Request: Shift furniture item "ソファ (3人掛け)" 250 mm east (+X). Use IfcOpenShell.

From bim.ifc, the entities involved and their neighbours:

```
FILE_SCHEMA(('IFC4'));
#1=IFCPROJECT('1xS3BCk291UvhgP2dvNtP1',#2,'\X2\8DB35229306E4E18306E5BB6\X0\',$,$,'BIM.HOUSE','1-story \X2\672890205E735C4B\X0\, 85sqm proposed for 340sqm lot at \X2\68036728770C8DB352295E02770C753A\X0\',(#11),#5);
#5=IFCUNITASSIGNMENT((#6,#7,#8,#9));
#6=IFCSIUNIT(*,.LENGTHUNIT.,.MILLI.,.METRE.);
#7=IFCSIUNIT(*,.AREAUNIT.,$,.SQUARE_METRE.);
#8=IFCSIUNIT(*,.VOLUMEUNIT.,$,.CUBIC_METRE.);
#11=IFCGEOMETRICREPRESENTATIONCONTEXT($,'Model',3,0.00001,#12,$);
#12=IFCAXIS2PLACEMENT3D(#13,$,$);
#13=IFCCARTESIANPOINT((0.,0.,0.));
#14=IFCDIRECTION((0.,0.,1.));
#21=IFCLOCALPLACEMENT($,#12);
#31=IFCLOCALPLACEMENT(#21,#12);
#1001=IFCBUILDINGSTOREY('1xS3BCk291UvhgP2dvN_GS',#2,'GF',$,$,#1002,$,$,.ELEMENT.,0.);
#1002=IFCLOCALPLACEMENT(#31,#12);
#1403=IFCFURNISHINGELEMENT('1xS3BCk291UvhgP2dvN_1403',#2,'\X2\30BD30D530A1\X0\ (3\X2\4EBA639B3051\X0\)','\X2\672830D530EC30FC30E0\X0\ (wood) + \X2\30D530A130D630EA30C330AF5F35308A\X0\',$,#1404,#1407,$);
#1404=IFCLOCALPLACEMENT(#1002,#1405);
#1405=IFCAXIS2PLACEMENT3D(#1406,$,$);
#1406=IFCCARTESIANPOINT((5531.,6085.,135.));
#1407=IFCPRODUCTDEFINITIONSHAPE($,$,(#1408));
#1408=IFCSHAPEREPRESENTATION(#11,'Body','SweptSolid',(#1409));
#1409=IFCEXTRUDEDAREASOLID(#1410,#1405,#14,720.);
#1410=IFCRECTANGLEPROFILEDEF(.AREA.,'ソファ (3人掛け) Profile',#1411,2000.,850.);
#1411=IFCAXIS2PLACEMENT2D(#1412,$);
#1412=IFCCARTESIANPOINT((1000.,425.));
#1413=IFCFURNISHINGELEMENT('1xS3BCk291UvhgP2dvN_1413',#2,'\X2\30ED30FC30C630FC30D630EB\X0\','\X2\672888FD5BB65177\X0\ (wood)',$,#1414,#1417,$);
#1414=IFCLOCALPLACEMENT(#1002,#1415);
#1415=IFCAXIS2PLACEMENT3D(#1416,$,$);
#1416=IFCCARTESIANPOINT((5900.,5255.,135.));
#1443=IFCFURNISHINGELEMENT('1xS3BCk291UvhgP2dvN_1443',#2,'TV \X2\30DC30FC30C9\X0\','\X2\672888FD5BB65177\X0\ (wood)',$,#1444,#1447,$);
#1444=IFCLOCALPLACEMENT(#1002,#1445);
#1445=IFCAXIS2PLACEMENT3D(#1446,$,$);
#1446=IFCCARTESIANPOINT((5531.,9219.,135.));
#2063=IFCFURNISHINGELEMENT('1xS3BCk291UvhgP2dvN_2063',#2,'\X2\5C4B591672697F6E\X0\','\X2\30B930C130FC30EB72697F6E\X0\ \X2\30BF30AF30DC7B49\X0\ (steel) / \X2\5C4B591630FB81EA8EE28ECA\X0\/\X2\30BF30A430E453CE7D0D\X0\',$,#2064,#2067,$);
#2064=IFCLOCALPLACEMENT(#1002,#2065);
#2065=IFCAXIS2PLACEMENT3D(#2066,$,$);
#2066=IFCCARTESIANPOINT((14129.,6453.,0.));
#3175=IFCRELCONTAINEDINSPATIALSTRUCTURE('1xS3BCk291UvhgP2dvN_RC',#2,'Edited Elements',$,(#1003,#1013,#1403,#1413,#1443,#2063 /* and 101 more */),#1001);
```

```python
import ifcopenshell
import ifcopenshell.api.geometry
import ifcopenshell.util.placement

model = ifcopenshell.open("bim.ifc")

item = model.by_guid("1xS3BCk291UvhgP2dvN_1403")
matrix = ifcopenshell.util.placement.get_local_placement(item.ObjectPlacement)
matrix[0, 3] += 250.0
ifcopenshell.api.geometry.edit_object_placement(model, product=item, matrix=matrix, is_si=False)

print(ifcopenshell.util.placement.get_local_placement(item.ObjectPlacement).round(3) + 0.0)

model.write("bim_rev.ifc")
```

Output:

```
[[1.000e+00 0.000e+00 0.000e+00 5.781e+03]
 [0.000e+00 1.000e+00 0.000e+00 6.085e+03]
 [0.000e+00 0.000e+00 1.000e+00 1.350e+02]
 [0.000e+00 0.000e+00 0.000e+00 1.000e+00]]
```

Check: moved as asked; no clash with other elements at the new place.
